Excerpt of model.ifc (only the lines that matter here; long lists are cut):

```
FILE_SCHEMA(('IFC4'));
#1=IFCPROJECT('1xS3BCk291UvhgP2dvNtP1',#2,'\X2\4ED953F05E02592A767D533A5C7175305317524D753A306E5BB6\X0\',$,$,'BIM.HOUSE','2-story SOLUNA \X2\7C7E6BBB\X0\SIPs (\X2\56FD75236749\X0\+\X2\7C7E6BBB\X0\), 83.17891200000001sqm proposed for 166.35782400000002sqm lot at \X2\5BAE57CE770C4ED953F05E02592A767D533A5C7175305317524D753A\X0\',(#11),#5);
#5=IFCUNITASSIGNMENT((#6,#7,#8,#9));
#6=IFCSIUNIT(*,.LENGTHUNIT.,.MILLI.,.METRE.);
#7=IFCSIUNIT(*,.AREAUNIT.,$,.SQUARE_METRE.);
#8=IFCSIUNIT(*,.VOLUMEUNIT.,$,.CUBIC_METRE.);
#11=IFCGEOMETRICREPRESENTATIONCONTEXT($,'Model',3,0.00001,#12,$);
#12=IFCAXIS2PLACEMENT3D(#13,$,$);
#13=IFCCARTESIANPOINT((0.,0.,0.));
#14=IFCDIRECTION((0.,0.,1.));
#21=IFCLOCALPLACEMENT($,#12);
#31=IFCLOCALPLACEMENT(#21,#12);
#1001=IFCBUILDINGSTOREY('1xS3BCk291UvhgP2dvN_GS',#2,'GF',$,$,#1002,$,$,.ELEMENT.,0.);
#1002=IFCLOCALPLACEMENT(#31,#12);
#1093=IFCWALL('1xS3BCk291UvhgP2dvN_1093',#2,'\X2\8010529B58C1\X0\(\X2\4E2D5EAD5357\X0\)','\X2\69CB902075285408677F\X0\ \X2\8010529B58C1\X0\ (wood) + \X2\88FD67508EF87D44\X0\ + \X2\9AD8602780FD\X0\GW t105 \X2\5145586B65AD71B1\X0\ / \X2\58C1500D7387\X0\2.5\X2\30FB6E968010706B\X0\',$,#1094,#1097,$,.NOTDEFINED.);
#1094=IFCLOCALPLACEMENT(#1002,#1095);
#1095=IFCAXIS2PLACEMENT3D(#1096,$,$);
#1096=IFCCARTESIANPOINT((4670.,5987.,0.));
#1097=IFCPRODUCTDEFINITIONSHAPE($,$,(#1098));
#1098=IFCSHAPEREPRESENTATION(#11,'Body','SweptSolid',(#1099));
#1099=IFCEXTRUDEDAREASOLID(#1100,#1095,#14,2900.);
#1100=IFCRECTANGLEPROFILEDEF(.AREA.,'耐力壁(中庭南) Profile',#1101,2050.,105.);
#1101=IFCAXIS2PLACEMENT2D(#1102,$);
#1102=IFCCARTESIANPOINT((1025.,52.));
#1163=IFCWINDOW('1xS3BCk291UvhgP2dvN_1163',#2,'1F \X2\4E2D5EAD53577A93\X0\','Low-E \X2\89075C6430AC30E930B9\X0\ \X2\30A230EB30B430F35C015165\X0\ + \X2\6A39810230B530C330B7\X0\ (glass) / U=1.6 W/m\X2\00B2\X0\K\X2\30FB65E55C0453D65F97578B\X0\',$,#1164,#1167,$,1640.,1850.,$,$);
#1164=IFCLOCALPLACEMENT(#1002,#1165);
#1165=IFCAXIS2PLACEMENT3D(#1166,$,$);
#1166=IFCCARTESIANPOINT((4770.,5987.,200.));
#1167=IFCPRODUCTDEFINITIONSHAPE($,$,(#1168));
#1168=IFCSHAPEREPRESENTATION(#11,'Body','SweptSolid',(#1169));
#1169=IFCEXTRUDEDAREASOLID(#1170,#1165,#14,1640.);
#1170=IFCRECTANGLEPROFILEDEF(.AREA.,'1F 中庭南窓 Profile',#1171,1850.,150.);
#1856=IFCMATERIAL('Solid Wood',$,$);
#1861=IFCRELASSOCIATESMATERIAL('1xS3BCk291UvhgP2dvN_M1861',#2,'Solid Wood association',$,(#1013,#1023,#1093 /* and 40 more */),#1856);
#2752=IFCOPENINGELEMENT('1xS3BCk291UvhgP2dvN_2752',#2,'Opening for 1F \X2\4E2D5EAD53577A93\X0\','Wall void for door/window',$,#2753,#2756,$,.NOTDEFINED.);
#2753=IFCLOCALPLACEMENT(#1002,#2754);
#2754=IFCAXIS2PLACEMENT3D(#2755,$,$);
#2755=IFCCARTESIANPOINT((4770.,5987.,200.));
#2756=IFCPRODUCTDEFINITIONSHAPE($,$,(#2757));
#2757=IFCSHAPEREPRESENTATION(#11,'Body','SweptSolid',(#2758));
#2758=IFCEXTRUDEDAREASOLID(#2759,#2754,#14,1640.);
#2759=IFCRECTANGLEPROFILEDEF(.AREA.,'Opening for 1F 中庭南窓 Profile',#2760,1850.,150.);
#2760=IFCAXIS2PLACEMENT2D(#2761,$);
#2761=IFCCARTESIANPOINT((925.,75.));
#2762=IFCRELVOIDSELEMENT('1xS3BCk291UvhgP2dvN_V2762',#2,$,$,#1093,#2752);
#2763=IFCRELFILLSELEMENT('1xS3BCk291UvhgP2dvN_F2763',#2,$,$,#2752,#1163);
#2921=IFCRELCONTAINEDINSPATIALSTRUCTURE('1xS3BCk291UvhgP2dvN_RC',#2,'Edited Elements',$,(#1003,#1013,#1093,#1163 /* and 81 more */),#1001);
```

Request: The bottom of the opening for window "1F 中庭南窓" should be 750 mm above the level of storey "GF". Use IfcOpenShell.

```python
import numpy as np
import ifcopenshell
import ifcopenshell.api.geometry
import ifcopenshell.geom
import ifcopenshell.util.element
import ifcopenshell.util.placement
import ifcopenshell.util.shape
import ifcopenshell.util.unit

model = ifcopenshell.open("model.ifc")
unit_scale = ifcopenshell.util.unit.calculate_unit_scale(model)

window = model.by_guid("1xS3BCk291UvhgP2dvN_1163")
opening = window.FillsVoids[0].RelatingOpeningElement
storey = ifcopenshell.util.element.get_container(window, ifc_class="IfcBuildingStorey")
level = ifcopenshell.util.placement.get_local_placement(storey.ObjectPlacement)[2, 3]

# The opening's origin need not be at the sill, so measure its lowest point.
shape = ifcopenshell.geom.create_shape(ifcopenshell.geom.settings(), opening)
bottom = ifcopenshell.util.shape.get_shape_bottom_elevation(shape, shape.geometry) / unit_scale
dz = level + 0.75 / unit_scale - bottom

shift = np.array([0.0, 0.0, dz])
# The window is not placed relative to its opening, so move both.
for product in (opening, window):
    matrix = ifcopenshell.util.placement.get_local_placement(product.ObjectPlacement)
    matrix[:3, 3] += shift
    ifcopenshell.api.geometry.edit_object_placement(model, product=product, matrix=matrix, is_si=False)

print(f"moved by {dz * unit_scale:+.3f} m")

model.write("model_edited.ifc")
```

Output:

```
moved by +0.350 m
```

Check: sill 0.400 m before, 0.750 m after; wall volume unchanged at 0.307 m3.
